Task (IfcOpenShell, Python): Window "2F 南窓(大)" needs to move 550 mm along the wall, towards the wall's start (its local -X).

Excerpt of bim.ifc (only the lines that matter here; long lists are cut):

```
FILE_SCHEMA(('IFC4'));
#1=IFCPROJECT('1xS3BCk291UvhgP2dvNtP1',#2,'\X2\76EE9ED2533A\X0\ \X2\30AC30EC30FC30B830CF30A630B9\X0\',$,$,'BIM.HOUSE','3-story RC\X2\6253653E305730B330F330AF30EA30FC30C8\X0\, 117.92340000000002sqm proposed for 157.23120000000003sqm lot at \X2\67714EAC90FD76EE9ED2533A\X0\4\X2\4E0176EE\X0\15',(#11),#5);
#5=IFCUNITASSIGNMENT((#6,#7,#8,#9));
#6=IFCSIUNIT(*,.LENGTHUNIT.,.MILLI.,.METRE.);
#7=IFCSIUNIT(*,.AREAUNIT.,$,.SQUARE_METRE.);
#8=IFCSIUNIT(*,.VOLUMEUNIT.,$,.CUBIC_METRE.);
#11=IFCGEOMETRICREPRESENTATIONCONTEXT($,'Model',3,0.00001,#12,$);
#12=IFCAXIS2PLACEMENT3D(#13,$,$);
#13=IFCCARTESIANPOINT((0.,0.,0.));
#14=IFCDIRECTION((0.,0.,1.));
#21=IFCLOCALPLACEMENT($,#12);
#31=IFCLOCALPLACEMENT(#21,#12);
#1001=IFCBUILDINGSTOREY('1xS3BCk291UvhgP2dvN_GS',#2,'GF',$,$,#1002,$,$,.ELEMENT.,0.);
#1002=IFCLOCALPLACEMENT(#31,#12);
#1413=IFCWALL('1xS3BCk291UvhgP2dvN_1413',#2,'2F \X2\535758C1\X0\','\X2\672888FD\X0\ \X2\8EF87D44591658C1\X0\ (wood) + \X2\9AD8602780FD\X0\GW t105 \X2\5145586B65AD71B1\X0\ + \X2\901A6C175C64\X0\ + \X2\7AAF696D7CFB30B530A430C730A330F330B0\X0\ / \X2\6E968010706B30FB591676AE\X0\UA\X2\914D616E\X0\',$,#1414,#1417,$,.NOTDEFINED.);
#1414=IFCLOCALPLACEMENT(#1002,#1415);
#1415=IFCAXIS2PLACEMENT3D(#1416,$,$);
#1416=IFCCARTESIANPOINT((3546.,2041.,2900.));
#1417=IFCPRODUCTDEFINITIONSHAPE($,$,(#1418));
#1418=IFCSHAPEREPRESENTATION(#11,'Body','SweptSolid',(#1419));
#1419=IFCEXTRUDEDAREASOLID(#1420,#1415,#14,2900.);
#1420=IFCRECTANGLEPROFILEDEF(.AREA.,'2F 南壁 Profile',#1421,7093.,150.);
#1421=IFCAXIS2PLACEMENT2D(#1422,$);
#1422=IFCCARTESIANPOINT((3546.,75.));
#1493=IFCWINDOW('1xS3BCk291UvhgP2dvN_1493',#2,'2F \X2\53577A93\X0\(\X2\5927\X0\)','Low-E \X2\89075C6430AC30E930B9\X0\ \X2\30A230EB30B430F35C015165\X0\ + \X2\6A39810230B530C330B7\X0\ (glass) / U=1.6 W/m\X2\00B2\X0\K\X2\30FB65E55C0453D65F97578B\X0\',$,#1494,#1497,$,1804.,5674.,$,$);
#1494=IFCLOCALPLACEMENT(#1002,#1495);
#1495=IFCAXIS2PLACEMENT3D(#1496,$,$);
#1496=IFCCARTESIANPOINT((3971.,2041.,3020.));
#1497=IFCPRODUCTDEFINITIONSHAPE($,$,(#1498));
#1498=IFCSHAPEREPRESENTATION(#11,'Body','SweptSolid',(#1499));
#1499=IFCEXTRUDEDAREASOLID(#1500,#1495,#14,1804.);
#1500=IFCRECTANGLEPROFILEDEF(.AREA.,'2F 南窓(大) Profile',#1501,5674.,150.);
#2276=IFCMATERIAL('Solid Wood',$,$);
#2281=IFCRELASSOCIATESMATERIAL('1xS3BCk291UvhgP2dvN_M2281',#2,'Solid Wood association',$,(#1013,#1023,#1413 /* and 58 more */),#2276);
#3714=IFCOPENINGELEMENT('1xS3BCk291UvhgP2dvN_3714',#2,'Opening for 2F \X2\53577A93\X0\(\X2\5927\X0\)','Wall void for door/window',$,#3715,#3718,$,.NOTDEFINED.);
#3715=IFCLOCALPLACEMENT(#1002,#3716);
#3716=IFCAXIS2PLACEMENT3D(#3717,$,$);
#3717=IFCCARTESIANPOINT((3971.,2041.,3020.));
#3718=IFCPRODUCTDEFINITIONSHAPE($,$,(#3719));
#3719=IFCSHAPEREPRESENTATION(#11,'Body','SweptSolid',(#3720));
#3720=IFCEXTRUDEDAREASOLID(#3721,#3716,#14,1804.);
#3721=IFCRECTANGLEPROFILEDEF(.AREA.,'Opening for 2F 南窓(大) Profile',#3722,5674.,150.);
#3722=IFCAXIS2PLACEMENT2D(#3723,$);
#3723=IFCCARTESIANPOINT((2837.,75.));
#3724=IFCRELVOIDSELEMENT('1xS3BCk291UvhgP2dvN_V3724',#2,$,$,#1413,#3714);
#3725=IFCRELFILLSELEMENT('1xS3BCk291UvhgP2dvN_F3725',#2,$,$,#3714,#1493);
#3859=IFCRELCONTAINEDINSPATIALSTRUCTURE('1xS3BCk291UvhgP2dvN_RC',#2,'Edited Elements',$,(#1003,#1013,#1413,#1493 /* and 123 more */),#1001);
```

```python
import ifcopenshell
import ifcopenshell.api.geometry
import ifcopenshell.util.placement

model = ifcopenshell.open("bim.ifc")

window = model.by_guid("1xS3BCk291UvhgP2dvN_1493")
opening = window.FillsVoids[0].RelatingOpeningElement
wall = opening.VoidsElements[0].RelatingBuildingElement

wall_matrix = ifcopenshell.util.placement.get_local_placement(wall.ObjectPlacement)
shift = wall_matrix[:3, 0] * -550.0
before = ifcopenshell.util.placement.get_local_placement(window.ObjectPlacement)[:3, 3].copy()

# The window is not placed relative to its opening, so move both.
for product in (opening, window):
    matrix = ifcopenshell.util.placement.get_local_placement(product.ObjectPlacement)
    matrix[:3, 3] += shift
    ifcopenshell.api.geometry.edit_object_placement(model, product=product, matrix=matrix, is_si=False)

after = ifcopenshell.util.placement.get_local_placement(window.ObjectPlacement)[:3, 3]
print("window moved by", (after - before).round(3) + 0.0)

model.write("bim_edited.ifc")
```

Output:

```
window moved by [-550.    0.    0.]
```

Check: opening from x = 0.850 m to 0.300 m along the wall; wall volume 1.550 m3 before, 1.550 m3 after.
